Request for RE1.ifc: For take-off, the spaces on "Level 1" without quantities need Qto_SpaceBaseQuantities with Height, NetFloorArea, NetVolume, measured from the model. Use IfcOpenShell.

First a look at what the model holds.

```python
import ifcopenshell
import ifcopenshell.util.element
import ifcopenshell.util.unit

model = ifcopenshell.open("RE1.ifc")
print(model.schema)
for unit_type in ("LENGTHUNIT", "AREAUNIT", "VOLUMEUNIT"):
    print(unit_type, ifcopenshell.util.unit.calculate_unit_scale(model, unit_type))
storey = next(s for s in model.by_type("IfcBuildingStorey") if s.Name == "Level 1")
spaces = [e for e in ifcopenshell.util.element.get_decomposition(storey) if e.is_a("IfcSpace")]
for e in sorted(spaces, key=lambda e: e.id()):
    print(e.id(), e.is_a(), e.Name, list(ifcopenshell.util.element.get_psets(e, qtos_only=True)), sep=" | ")
```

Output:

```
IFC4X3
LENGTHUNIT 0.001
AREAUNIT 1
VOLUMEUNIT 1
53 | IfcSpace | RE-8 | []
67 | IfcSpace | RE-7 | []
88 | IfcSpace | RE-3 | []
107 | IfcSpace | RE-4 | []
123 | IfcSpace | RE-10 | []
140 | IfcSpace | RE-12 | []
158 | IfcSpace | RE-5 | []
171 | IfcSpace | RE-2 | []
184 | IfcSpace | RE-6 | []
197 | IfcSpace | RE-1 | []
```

```python
import ifcopenshell
import ifcopenshell.api.pset
import ifcopenshell.geom
import ifcopenshell.util.element
import ifcopenshell.util.shape
import ifcopenshell.util.unit

model = ifcopenshell.open("RE1.ifc")
unit_scale = ifcopenshell.util.unit.calculate_unit_scale(model)
area_scale = ifcopenshell.util.unit.calculate_unit_scale(model, "AREAUNIT")
volume_scale = ifcopenshell.util.unit.calculate_unit_scale(model, "VOLUMEUNIT")
settings = ifcopenshell.geom.settings()

storey = next(s for s in model.by_type("IfcBuildingStorey") if s.Name == "Level 1")
spaces = [e for e in ifcopenshell.util.element.get_decomposition(storey) if e.is_a("IfcSpace")]

for e in sorted(spaces, key=lambda e: e.id()):
    if ifcopenshell.util.element.get_psets(e, qtos_only=True, should_inherit=False):
        continue
    # Geometry comes back in metres, in the element's own axes.
    shape = ifcopenshell.geom.create_shape(settings, e)
    values = {
        "Height": ifcopenshell.util.shape.get_z(shape.geometry) / unit_scale,
        "NetFloorArea": ifcopenshell.util.shape.get_footprint_area(shape.geometry) / area_scale,
        "NetVolume": ifcopenshell.util.shape.get_volume(shape.geometry) / volume_scale,
    }
    qto = ifcopenshell.api.pset.add_qto(model, product=e, name="Qto_SpaceBaseQuantities")
    ifcopenshell.api.pset.edit_qto(model, qto=qto, properties=values)
    print(e.id(), {k: round(v, 3) for k, v in values.items()})

model.write("RE1-out.ifc")
```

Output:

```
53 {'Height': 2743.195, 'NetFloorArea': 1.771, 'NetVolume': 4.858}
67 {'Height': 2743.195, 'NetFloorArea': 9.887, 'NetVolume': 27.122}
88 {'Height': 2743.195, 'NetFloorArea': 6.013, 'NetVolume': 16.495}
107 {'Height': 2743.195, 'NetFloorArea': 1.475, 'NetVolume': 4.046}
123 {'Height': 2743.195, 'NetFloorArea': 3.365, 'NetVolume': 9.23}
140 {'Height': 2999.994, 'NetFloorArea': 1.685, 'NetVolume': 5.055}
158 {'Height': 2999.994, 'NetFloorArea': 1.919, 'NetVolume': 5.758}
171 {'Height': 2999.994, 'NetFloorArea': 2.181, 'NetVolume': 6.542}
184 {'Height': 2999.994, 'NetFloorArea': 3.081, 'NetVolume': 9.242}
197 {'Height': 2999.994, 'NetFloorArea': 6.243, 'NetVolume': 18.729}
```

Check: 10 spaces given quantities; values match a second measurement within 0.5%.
